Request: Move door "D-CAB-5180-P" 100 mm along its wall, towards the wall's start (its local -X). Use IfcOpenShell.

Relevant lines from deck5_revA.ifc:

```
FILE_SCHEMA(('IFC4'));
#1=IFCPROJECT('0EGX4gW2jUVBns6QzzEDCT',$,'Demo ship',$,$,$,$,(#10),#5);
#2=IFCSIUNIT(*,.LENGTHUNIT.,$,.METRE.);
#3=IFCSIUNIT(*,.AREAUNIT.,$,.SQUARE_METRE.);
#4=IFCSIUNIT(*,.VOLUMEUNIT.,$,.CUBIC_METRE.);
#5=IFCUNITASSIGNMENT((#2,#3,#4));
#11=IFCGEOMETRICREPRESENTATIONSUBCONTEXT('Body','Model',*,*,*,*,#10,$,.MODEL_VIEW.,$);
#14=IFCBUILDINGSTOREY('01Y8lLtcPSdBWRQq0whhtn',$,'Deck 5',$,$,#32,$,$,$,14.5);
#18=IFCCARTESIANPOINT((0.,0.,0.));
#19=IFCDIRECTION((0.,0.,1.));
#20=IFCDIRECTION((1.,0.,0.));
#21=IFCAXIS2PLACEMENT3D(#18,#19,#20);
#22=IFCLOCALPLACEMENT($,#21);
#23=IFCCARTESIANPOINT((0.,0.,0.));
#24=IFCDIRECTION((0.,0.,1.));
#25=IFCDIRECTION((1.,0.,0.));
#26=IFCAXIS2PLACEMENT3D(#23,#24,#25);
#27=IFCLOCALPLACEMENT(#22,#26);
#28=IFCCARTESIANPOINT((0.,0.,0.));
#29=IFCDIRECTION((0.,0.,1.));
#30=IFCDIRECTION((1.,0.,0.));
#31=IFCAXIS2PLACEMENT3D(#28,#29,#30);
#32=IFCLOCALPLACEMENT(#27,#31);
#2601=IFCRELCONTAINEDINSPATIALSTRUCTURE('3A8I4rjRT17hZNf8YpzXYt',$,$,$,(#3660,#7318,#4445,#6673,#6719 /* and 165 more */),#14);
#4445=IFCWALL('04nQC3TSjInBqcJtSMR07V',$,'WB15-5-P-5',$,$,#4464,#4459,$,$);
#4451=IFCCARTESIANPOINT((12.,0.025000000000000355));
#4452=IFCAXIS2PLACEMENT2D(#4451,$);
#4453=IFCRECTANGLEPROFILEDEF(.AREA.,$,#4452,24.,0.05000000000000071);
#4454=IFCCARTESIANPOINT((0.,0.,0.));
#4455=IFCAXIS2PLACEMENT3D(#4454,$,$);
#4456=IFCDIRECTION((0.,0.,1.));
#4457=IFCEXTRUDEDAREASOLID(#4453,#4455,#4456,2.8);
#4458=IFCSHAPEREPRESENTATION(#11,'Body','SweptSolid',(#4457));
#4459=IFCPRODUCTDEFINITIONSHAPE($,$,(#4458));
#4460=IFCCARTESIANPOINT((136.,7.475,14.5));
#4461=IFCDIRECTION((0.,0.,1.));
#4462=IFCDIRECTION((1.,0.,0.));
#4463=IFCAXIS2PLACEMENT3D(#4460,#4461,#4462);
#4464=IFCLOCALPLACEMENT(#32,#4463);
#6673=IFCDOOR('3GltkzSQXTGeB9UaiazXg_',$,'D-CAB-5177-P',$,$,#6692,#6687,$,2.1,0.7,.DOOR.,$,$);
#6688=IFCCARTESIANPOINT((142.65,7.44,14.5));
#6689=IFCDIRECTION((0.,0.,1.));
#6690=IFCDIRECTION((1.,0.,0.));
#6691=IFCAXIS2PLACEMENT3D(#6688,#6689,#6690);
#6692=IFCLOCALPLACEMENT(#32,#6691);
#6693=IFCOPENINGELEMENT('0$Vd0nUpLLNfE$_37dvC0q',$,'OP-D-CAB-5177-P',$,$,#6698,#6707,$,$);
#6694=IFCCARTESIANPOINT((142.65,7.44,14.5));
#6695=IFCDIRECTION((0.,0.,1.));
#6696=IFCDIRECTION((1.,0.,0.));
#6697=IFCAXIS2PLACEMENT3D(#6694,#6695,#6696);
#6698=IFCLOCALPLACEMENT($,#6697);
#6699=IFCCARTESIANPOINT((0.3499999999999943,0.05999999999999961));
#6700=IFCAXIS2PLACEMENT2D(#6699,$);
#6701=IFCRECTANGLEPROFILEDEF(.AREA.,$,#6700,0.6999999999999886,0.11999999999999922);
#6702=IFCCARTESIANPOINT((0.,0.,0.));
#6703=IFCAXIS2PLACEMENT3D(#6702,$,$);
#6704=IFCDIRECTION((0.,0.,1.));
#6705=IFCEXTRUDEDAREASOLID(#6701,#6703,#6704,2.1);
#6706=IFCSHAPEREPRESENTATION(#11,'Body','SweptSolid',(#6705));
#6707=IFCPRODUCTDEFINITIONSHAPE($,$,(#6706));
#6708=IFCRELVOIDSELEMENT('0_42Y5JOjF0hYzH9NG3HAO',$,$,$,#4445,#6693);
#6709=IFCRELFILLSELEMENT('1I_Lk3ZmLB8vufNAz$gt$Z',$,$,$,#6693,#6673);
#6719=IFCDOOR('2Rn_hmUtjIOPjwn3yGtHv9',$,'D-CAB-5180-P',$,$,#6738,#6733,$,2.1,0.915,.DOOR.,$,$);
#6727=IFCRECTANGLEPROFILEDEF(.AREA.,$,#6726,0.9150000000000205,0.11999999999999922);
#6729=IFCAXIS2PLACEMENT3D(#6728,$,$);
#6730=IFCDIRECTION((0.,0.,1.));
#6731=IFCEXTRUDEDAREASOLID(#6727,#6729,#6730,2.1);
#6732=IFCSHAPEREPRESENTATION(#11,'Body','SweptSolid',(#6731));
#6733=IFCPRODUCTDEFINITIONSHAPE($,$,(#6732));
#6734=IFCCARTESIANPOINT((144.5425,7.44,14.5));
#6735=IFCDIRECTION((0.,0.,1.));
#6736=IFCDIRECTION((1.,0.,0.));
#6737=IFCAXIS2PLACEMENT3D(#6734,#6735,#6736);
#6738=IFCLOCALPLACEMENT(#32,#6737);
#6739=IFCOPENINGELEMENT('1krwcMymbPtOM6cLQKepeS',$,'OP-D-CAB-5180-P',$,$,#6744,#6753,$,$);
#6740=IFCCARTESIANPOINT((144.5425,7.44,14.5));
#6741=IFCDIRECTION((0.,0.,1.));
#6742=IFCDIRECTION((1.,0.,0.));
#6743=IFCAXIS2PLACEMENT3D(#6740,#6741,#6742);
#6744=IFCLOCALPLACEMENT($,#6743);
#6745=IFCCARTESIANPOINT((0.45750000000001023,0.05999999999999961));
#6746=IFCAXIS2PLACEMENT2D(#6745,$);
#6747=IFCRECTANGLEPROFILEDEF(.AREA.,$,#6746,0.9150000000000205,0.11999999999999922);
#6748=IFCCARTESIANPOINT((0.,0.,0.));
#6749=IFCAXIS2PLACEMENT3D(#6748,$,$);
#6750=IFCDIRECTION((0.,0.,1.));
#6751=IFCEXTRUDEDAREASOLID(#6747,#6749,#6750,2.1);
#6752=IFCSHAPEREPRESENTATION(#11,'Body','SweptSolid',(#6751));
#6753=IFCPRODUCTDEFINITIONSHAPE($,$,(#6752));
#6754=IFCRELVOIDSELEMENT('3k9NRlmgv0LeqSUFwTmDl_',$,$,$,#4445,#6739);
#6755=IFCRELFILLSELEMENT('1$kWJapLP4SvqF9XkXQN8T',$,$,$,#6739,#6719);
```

```python
import ifcopenshell
import ifcopenshell.api.geometry
import ifcopenshell.util.placement

model = ifcopenshell.open("deck5_revA.ifc")

door = model.by_guid("2Rn_hmUtjIOPjwn3yGtHv9")
opening = door.FillsVoids[0].RelatingOpeningElement
wall = opening.VoidsElements[0].RelatingBuildingElement

wall_matrix = ifcopenshell.util.placement.get_local_placement(wall.ObjectPlacement)
shift = wall_matrix[:3, 0] * -0.1
before = ifcopenshell.util.placement.get_local_placement(door.ObjectPlacement)[:3, 3].copy()

# The door is not placed relative to its opening, so move both.
for product in (opening, door):
    matrix = ifcopenshell.util.placement.get_local_placement(product.ObjectPlacement)
    matrix[:3, 3] += shift
    ifcopenshell.api.geometry.edit_object_placement(model, product=product, matrix=matrix, is_si=False)

after = ifcopenshell.util.placement.get_local_placement(door.ObjectPlacement)[:3, 3]
print("door moved by", (after - before).round(3) + 0.0)

model.write("deck5_revA-out.ifc")
```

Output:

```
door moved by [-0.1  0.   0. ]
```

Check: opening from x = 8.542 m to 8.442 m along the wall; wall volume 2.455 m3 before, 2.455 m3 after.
